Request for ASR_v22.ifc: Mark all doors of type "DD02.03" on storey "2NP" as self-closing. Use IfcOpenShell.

First a look at what the model holds.

```python
import ifcopenshell
import ifcopenshell.util.element

model = ifcopenshell.open("ASR_v22.ifc")
print(model.schema)
storey = next(s for s in model.by_type("IfcBuildingStorey") if s.Name == "2NP")
doors = [e for e in ifcopenshell.util.element.get_decomposition(storey) if e.is_a("IfcDoor")]
seen = {}
for e in doors:
    element_type = ifcopenshell.util.element.get_type(e)
    key = (element_type.Name if element_type != e and element_type else None, ifcopenshell.util.element.get_pset(e, "Pset_DoorCommon", "SelfClosing"))
    seen[key] = seen.get(key, 0) + 1
for (name, value), count in sorted(seen.items(), key=str):
    print(count, "x", name, "|", value)
```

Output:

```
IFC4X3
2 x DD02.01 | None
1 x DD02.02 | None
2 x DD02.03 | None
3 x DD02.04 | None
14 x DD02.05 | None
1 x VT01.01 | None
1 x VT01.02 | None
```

```python
import ifcopenshell
import ifcopenshell.api.pset
import ifcopenshell.util.element

model = ifcopenshell.open("ASR_v22.ifc")

storey = next(s for s in model.by_type("IfcBuildingStorey") if s.Name == "2NP")
doors = [e for e in ifcopenshell.util.element.get_decomposition(storey) if e.is_a("IfcDoor")]

count = 0
for e in doors:
    element_type = ifcopenshell.util.element.get_type(e)
    if element_type in (None, e) or element_type.Name != "DD02.03":
        continue
    # add_pset returns the element's existing set when there is one.
    pset = ifcopenshell.api.pset.add_pset(model, product=e, name="Pset_DoorCommon")
    ifcopenshell.api.pset.edit_pset(model, pset=pset, properties={"SelfClosing": True})
    count += 1

print(count, "doors updated")

model.write("ASR_v22_v2.ifc")
```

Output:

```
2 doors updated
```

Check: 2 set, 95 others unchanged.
